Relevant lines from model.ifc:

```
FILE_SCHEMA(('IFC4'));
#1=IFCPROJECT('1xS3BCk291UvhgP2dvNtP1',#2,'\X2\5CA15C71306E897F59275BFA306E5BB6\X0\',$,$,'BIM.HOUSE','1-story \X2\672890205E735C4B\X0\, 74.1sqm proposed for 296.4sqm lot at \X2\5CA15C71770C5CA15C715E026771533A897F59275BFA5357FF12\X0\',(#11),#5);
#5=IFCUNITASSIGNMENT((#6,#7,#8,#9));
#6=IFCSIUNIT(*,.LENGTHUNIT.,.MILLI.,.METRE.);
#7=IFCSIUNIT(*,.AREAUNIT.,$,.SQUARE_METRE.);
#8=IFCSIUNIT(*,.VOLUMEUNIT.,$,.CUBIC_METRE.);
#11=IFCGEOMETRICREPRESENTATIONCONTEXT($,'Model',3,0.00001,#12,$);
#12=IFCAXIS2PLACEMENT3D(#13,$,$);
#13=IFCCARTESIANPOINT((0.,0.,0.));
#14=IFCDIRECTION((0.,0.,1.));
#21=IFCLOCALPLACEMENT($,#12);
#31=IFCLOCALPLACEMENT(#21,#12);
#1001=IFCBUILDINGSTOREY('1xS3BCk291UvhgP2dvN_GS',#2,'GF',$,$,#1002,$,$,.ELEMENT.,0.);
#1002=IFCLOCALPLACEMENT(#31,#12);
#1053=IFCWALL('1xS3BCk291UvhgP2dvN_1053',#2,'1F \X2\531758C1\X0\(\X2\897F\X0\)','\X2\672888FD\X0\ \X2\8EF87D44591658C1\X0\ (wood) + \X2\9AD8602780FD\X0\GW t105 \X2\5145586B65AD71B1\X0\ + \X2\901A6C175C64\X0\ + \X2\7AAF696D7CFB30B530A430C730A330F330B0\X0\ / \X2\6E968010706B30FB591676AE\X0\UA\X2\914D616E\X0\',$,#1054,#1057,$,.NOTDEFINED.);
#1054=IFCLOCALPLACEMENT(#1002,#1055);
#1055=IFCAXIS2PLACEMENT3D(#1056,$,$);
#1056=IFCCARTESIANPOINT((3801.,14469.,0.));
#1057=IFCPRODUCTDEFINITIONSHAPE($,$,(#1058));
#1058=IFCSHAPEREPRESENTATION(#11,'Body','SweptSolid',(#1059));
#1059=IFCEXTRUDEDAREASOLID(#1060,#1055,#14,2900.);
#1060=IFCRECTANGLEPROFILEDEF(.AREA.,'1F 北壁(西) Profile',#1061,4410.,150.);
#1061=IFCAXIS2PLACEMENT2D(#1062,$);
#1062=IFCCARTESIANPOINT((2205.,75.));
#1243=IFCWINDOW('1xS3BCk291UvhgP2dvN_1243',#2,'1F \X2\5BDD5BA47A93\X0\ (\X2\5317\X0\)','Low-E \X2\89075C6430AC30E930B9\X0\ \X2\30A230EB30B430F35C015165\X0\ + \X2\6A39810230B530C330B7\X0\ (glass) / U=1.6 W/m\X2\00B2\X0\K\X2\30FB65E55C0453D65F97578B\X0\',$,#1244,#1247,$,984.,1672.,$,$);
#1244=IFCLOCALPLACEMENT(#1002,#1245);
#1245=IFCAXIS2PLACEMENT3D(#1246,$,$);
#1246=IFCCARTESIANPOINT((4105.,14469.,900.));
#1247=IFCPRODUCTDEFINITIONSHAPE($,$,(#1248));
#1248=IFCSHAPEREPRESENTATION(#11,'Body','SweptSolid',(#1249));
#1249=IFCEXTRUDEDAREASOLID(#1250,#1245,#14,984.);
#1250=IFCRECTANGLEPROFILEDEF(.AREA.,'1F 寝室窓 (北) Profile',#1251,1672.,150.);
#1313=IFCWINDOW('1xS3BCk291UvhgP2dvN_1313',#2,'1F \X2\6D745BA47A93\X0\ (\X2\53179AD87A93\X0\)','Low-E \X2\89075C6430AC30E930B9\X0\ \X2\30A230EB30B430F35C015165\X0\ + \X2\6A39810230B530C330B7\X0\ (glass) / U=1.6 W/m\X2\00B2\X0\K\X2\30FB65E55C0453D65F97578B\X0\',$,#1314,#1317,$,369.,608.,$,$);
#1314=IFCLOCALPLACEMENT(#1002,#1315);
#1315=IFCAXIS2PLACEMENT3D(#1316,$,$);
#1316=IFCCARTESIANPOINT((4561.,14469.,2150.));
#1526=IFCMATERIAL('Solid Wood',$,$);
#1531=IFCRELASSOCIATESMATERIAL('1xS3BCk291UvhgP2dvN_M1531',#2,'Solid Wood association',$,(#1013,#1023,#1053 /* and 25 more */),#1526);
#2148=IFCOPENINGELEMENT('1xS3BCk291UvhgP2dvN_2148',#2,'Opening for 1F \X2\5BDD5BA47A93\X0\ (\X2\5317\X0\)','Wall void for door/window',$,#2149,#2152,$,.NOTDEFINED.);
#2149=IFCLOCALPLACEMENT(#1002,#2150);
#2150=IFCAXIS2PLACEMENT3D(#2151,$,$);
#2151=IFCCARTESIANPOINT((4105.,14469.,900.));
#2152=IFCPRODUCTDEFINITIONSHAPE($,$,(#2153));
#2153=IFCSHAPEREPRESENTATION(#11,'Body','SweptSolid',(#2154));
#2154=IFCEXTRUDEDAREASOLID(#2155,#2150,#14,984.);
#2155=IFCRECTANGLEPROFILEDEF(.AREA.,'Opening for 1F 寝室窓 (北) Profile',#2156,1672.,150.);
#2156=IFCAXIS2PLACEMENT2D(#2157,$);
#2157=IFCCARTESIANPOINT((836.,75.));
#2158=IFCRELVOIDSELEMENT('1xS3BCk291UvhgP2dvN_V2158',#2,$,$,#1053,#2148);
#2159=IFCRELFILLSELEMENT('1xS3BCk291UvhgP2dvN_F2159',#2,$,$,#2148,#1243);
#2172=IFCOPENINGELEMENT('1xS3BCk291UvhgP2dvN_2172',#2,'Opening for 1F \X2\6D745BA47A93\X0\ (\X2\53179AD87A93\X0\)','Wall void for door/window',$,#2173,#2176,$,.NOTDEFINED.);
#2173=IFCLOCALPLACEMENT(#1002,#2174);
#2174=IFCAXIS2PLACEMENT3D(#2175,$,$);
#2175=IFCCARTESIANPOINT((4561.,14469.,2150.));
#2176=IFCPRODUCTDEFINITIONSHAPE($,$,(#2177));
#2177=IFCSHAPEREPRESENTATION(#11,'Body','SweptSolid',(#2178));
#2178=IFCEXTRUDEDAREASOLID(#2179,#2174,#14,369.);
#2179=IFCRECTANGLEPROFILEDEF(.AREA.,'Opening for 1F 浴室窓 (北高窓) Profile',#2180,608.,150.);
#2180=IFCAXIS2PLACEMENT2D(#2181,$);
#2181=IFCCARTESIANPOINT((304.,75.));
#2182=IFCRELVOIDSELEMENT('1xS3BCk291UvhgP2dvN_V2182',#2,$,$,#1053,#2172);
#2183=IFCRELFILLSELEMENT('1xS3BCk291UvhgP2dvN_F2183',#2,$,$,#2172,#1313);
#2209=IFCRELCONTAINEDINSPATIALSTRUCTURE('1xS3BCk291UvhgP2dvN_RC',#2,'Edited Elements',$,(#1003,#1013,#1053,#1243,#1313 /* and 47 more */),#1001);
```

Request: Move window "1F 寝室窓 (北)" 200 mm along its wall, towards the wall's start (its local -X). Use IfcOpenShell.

```python
import ifcopenshell
import ifcopenshell.api.geometry
import ifcopenshell.util.placement

model = ifcopenshell.open("model.ifc")

window = model.by_id(1243)
opening = window.FillsVoids[0].RelatingOpeningElement
wall = opening.VoidsElements[0].RelatingBuildingElement

wall_matrix = ifcopenshell.util.placement.get_local_placement(wall.ObjectPlacement)
shift = wall_matrix[:3, 0] * -200.0
before = ifcopenshell.util.placement.get_local_placement(window.ObjectPlacement)[:3, 3].copy()

# The window is not placed relative to its opening, so move both.
for product in (opening, window):
    matrix = ifcopenshell.util.placement.get_local_placement(product.ObjectPlacement)
    matrix[:3, 3] += shift
    ifcopenshell.api.geometry.edit_object_placement(model, product=product, matrix=matrix, is_si=False)

after = ifcopenshell.util.placement.get_local_placement(window.ObjectPlacement)[:3, 3]
print("window moved by", (after - before).round(3) + 0.0)

model.write("model_v2.ifc")
```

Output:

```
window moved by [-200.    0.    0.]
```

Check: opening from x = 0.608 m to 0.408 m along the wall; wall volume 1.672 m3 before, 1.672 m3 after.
